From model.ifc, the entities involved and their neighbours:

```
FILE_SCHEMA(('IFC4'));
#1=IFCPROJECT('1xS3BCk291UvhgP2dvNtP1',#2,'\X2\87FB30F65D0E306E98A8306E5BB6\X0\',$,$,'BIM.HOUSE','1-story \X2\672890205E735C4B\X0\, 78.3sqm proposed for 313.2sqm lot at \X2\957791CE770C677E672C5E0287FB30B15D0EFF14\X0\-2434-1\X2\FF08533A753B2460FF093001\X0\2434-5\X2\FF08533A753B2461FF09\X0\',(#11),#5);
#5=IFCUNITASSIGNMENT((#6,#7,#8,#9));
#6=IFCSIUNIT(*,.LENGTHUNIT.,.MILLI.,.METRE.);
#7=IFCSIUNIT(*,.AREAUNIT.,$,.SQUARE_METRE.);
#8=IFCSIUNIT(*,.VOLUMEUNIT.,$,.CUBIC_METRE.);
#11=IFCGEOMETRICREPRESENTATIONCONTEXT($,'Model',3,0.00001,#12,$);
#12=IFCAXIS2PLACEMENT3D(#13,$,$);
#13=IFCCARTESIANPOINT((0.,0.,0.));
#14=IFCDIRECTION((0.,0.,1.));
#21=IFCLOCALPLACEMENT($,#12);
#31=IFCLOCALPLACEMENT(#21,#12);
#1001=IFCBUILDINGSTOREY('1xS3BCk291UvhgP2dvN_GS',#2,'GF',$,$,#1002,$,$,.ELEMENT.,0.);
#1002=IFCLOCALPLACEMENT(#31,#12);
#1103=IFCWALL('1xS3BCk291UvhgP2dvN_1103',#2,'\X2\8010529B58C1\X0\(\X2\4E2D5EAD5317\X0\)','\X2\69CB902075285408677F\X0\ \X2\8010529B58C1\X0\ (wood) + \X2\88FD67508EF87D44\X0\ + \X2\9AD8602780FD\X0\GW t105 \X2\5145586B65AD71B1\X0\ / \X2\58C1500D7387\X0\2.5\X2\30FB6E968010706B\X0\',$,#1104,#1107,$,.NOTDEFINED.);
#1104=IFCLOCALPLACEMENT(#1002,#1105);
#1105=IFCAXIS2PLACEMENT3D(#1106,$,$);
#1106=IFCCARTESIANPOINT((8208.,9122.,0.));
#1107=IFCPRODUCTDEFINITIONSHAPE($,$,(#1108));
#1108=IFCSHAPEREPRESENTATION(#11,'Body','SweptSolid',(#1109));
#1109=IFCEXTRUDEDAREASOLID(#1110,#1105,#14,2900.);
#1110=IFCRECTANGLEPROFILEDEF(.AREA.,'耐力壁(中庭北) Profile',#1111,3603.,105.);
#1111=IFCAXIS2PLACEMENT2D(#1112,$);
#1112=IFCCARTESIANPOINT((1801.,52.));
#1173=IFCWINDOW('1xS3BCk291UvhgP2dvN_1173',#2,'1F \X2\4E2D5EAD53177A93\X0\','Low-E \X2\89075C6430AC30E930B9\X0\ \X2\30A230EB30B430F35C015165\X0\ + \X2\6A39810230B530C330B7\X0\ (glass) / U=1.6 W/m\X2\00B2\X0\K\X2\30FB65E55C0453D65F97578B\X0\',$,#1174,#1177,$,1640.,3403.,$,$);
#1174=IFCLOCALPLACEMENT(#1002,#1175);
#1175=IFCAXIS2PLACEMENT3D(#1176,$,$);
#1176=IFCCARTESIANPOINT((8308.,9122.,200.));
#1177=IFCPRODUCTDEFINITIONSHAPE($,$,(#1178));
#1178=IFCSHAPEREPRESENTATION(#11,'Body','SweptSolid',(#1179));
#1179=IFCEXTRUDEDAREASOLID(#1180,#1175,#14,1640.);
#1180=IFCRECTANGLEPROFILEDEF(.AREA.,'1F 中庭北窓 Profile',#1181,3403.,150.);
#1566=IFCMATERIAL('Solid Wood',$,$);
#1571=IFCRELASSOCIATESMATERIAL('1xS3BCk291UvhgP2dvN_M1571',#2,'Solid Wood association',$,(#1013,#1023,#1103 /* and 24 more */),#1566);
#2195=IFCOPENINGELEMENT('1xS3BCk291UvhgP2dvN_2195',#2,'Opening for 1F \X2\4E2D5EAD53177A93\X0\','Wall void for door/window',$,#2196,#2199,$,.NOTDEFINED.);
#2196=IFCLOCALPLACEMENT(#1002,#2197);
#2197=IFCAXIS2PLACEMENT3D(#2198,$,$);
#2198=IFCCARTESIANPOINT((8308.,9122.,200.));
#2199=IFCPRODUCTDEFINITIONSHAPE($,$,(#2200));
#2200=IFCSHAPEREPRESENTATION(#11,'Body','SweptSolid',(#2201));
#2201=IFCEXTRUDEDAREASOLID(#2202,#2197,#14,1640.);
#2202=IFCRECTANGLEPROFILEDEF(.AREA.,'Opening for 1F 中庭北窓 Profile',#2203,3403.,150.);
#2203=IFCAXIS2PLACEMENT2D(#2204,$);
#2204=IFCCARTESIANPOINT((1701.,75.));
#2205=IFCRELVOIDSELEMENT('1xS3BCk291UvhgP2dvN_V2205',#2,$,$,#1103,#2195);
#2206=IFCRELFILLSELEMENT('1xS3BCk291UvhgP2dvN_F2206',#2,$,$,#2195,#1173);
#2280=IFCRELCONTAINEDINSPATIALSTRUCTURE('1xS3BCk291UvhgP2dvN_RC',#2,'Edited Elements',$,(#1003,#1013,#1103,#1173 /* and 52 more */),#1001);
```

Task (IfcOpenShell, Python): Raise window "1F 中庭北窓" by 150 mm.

```python
import numpy as np
import ifcopenshell
import ifcopenshell.api.geometry
import ifcopenshell.util.placement
import ifcopenshell.util.unit

model = ifcopenshell.open("model.ifc")
unit_scale = ifcopenshell.util.unit.calculate_unit_scale(model)

window = model.by_guid("1xS3BCk291UvhgP2dvN_1173")
opening = window.FillsVoids[0].RelatingOpeningElement
dz = 150.0

shift = np.array([0.0, 0.0, dz])
# The window is not placed relative to its opening, so move both.
for product in (opening, window):
    matrix = ifcopenshell.util.placement.get_local_placement(product.ObjectPlacement)
    matrix[:3, 3] += shift
    ifcopenshell.api.geometry.edit_object_placement(model, product=product, matrix=matrix, is_si=False)

print(f"moved by {dz * unit_scale:+.3f} m")

model.write("model_rev.ifc")
```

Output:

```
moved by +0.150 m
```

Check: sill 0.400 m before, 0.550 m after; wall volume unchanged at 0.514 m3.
